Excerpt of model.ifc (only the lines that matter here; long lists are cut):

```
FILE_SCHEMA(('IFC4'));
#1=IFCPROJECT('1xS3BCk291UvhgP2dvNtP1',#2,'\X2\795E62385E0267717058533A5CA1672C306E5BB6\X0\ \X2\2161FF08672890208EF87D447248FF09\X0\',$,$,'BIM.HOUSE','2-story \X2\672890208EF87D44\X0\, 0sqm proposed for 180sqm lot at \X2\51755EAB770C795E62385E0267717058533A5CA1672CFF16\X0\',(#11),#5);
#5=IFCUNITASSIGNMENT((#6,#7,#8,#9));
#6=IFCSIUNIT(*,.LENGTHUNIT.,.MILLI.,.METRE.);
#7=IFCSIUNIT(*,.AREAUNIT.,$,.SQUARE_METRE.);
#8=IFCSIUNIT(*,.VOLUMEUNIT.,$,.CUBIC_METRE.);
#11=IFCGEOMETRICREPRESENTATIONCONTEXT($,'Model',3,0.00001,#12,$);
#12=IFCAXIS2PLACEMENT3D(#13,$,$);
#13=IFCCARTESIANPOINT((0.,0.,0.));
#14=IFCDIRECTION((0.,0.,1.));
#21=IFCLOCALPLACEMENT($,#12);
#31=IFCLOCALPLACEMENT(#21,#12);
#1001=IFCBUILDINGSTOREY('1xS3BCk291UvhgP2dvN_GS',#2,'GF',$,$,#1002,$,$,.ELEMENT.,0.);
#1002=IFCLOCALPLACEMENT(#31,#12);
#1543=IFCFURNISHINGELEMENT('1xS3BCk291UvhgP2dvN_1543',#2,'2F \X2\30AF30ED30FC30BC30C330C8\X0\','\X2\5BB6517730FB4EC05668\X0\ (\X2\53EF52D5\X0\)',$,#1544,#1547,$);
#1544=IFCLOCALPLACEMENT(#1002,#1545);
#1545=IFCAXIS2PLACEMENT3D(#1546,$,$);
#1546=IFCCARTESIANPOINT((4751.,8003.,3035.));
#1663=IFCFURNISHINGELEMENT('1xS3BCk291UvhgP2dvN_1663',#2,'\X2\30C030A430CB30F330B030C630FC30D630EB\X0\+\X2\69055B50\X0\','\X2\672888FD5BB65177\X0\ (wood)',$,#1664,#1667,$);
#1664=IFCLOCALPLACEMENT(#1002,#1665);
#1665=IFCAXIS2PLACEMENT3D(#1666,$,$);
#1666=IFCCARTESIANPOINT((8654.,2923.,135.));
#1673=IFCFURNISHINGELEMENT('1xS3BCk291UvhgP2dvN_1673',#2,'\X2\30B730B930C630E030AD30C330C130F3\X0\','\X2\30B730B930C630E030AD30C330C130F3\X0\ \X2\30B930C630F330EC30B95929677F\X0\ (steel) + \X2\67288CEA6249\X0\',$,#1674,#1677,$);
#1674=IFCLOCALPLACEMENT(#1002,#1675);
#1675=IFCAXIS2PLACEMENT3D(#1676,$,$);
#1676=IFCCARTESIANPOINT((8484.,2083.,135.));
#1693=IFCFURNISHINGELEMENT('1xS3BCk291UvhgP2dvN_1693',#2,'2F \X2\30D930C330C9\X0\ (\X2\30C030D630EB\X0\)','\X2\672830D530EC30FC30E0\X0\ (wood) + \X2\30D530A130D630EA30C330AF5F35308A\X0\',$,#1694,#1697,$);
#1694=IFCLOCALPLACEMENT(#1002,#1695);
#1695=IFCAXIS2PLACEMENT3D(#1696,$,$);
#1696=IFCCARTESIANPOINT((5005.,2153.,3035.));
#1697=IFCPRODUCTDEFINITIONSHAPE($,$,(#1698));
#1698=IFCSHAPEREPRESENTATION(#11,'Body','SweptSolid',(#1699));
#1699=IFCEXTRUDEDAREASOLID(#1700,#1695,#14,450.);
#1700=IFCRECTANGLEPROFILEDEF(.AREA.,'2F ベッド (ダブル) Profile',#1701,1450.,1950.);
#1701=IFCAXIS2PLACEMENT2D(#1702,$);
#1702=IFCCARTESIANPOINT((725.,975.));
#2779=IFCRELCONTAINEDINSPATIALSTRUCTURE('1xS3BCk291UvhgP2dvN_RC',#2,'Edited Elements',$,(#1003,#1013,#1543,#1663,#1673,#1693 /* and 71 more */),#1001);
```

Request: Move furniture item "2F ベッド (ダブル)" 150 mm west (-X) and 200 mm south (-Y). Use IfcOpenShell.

```python
import ifcopenshell
import ifcopenshell.api.geometry
import ifcopenshell.util.placement

model = ifcopenshell.open("model.ifc")

item = model.by_id(1693)
matrix = ifcopenshell.util.placement.get_local_placement(item.ObjectPlacement)
matrix[0, 3] -= 150.0
matrix[1, 3] -= 200.0
ifcopenshell.api.geometry.edit_object_placement(model, product=item, matrix=matrix, is_si=False)

print(ifcopenshell.util.placement.get_local_placement(item.ObjectPlacement).round(3) + 0.0)

model.write("model_edited.ifc")
```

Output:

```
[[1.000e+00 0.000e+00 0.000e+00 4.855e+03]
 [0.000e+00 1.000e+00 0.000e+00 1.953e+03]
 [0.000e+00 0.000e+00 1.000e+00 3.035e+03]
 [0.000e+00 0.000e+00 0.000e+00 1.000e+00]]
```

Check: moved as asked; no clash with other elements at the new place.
